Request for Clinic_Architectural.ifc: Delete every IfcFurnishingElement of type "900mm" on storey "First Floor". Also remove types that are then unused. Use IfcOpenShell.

First a look at what the model holds.

```python
import ifcopenshell
import ifcopenshell.util.element

model = ifcopenshell.open("Clinic_Architectural.ifc")
print(model.schema)
storey = next(s for s in model.by_type("IfcBuildingStorey") if s.Name == "First Floor")
furniture = [e for e in ifcopenshell.util.element.get_decomposition(storey) if e.is_a("IfcFurnishingElement")]
seen = {}
for e in furniture:
    element_type = ifcopenshell.util.element.get_type(e)
    name = element_type.Name if element_type not in (None, e) else None
    seen[name] = seen.get(name, 0) + 1
for name, count in sorted(seen.items(), key=str):
    print(count, "x", name)
```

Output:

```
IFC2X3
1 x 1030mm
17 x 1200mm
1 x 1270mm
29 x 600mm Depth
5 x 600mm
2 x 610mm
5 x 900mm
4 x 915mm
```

```python
import ifcopenshell
import ifcopenshell.api.root
import ifcopenshell.util.element

model = ifcopenshell.open("Clinic_Architectural.ifc")

storey = next(s for s in model.by_type("IfcBuildingStorey") if s.Name == "First Floor")
furniture = [e for e in ifcopenshell.util.element.get_decomposition(storey) if e.is_a("IfcFurnishingElement")]
targets = [e for e in furniture if (t := ifcopenshell.util.element.get_type(e)) not in (None, e) and t.Name == "900mm"]
types = {ifcopenshell.util.element.get_type(e) for e in targets} - {None, *targets}

for e in targets:
    ifcopenshell.api.root.remove_product(model, product=e)
print(len(targets), "removed")

unused = [t for t in types if not ifcopenshell.util.element.get_types(t)]
for t in unused:
    ifcopenshell.api.root.remove_product(model, product=t)
print(len(unused), "unused types removed")

model.write("Clinic_Architectural-out.ifc")
```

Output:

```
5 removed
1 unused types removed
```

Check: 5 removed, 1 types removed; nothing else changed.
